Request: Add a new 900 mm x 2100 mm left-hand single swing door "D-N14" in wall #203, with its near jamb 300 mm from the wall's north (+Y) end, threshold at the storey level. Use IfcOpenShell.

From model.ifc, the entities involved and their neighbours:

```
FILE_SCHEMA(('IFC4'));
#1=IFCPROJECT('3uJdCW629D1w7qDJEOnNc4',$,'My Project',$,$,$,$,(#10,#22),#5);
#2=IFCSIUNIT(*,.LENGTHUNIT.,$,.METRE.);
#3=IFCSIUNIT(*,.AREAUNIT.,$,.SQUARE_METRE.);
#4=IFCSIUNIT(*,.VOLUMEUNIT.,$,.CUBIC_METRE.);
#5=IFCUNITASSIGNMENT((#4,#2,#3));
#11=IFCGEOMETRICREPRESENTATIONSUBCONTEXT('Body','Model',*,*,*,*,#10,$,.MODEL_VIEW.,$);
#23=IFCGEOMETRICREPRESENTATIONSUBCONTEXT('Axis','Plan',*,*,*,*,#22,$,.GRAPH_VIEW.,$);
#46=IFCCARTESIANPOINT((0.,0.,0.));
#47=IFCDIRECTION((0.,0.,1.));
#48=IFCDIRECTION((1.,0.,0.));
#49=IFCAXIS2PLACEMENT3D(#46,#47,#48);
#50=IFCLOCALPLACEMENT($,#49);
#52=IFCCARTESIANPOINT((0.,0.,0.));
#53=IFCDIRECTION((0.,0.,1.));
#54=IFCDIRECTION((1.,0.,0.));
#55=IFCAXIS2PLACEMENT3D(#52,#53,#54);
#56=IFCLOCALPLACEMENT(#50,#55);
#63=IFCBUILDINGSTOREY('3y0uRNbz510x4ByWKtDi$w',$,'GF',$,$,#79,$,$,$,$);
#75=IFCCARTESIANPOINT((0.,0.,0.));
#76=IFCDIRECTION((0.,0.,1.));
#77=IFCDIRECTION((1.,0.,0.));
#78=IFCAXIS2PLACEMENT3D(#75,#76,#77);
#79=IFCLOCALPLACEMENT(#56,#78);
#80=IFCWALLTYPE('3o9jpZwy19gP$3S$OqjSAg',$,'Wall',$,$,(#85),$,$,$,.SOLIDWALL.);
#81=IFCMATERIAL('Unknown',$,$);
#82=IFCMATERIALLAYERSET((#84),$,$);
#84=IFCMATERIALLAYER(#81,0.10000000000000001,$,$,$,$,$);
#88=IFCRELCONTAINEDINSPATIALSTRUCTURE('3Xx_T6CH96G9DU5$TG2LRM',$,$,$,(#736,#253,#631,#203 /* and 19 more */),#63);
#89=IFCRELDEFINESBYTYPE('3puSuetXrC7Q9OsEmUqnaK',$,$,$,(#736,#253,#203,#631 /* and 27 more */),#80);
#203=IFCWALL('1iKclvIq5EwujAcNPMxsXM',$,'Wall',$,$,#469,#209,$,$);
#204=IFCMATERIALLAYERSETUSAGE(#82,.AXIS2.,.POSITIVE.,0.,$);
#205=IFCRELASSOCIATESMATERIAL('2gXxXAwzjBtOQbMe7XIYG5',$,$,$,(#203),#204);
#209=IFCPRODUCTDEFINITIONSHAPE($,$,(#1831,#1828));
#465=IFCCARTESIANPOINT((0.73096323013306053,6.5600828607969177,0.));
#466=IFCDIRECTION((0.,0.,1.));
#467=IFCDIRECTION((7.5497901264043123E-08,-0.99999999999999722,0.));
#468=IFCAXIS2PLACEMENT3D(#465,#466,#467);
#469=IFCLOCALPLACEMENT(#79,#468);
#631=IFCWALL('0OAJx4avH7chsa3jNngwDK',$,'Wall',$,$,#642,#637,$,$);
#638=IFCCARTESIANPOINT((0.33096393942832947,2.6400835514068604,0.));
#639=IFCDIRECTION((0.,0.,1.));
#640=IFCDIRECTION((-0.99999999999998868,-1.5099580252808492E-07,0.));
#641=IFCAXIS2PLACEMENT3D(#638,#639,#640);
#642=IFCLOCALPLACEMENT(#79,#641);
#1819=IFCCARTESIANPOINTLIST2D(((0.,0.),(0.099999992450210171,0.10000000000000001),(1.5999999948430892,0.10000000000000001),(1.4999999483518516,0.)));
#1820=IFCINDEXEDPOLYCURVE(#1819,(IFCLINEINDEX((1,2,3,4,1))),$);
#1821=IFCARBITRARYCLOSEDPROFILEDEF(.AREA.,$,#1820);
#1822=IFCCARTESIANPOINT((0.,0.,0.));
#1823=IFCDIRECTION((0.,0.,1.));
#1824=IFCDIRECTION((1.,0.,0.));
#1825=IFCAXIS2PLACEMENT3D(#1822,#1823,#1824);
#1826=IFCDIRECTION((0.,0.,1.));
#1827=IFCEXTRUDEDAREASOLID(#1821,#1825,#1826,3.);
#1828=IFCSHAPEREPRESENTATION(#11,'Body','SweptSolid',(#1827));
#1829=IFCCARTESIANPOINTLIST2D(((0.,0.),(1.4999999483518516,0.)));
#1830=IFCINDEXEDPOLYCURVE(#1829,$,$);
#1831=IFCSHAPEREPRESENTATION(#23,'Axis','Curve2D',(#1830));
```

```python
import numpy as np
import ifcopenshell
import ifcopenshell.api.feature
import ifcopenshell.api.geometry
import ifcopenshell.api.root
import ifcopenshell.api.spatial
import ifcopenshell.geom
import ifcopenshell.util.element
import ifcopenshell.util.placement
import ifcopenshell.util.representation
import ifcopenshell.util.shape
import ifcopenshell.util.unit

model = ifcopenshell.open("model.ifc")
unit_scale = ifcopenshell.util.unit.calculate_unit_scale(model)
settings = ifcopenshell.geom.settings()


def volume(element):
    """Net volume in cubic metres, openings subtracted."""
    shape = ifcopenshell.geom.create_shape(settings, element)
    return ifcopenshell.util.shape.get_volume(shape.geometry)


wall = model.by_guid("1iKclvIq5EwujAcNPMxsXM")
storey = ifcopenshell.util.element.get_container(wall, ifc_class="IfcBuildingStorey")
context = ifcopenshell.util.representation.get_context(model, "Model", "Body", "MODEL_VIEW")
before = volume(wall)

width, height, from_end, sill = 0.9, 2.1, 0.3, 0.0  # metres

# The wall runs along its own X axis, and the end named is its -X end.
wall_shape = ifcopenshell.geom.create_shape(settings, wall)
x, y, z = ifcopenshell.util.shape.get_vertices(wall_shape.geometry).T
start = x.min() + from_end
face, thickness = float(y.min()), float(y.max() - y.min())
wall_matrix = ifcopenshell.util.placement.get_local_placement(wall.ObjectPlacement)
level = ifcopenshell.util.placement.get_local_placement(storey.ObjectPlacement)[2, 3]


def in_wall(x, y):
    """Placement at x, y metres in the wall's axes, at sill height."""
    matrix = wall_matrix.copy()
    matrix[:, 3] = wall_matrix @ np.array([x / unit_scale, y / unit_scale, 0.0, 1.0])
    matrix[2, 3] = level + sill / unit_scale
    return matrix


# Opening: a box that overshoots both wall faces by 50 mm.
opening = ifcopenshell.api.root.create_entity(model, ifc_class="IfcOpeningElement", predefined_type="OPENING")
box = ifcopenshell.api.geometry.add_wall_representation(
    model, context=context, length=width, height=height, thickness=thickness + 0.1
)
ifcopenshell.api.geometry.assign_representation(model, product=opening, representation=box)
ifcopenshell.api.geometry.edit_object_placement(model, product=opening, matrix=in_wall(start, face - 0.05), is_si=False)
ifcopenshell.api.feature.add_feature(model, feature=opening, element=wall)

door = ifcopenshell.api.root.create_entity(model, ifc_class="IfcDoor", name="D-N14", predefined_type="DOOR")
door.OverallWidth, door.OverallHeight = width / unit_scale, height / unit_scale
door.OperationType = "SINGLE_SWING_LEFT"
body = ifcopenshell.api.geometry.add_door_representation(
    model,
    context=context,
    overall_width=door.OverallWidth,
    overall_height=door.OverallHeight,
    operation_type="SINGLE_SWING_LEFT",
    lining_properties={"LiningDepth": thickness / unit_scale, "ThresholdDepth": thickness / unit_scale},
)
ifcopenshell.api.geometry.assign_representation(model, product=door, representation=body)
ifcopenshell.api.spatial.assign_container(model, products=[door], relating_structure=storey)
ifcopenshell.api.feature.add_filling(model, opening=opening, element=door)

# The lining spans the wall, so the door starts at the wall face.
ifcopenshell.api.geometry.edit_object_placement(model, product=door, matrix=in_wall(start, face), is_si=False)

after = volume(wall)

print(f"wall volume {before:.3f} -> {after:.3f} m3")

model.write("model_updated.ifc")
```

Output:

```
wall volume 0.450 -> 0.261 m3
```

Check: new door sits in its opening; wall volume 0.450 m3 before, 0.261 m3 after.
